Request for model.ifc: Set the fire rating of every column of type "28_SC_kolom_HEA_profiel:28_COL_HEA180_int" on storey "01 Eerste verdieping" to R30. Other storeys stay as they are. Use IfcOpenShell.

First a look at what the model holds.

```python
import ifcopenshell
import ifcopenshell.util.element

model = ifcopenshell.open("model.ifc")
print(model.schema)
storey = next(s for s in model.by_type("IfcBuildingStorey") if s.Name == "01 Eerste verdieping")
columns = [e for e in ifcopenshell.util.element.get_decomposition(storey) if e.is_a("IfcColumn")]
seen = {}
for e in columns:
    element_type = ifcopenshell.util.element.get_type(e)
    key = (element_type.Name if element_type != e and element_type else None, ifcopenshell.util.element.get_pset(e, "Pset_ColumnCommon", "FireRating"))
    seen[key] = seen.get(key, 0) + 1
for (name, value), count in sorted(seen.items(), key=str):
    print(count, "x", name, "|", value)
```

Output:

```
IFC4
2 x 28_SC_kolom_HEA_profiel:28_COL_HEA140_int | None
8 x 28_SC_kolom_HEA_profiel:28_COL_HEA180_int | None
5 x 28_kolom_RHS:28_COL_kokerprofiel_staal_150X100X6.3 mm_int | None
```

```python
import ifcopenshell
import ifcopenshell.api.pset
import ifcopenshell.util.element

model = ifcopenshell.open("model.ifc")

storey = next(s for s in model.by_type("IfcBuildingStorey") if s.Name == "01 Eerste verdieping")
columns = [e for e in ifcopenshell.util.element.get_decomposition(storey) if e.is_a("IfcColumn")]

count = 0
for e in columns:
    element_type = ifcopenshell.util.element.get_type(e)
    if element_type in (None, e) or element_type.Name != "28_SC_kolom_HEA_profiel:28_COL_HEA180_int":
        continue
    # add_pset returns the element's existing set when there is one.
    pset = ifcopenshell.api.pset.add_pset(model, product=e, name="Pset_ColumnCommon")
    ifcopenshell.api.pset.edit_pset(model, pset=pset, properties={"FireRating": "R30"})
    count += 1

print(count, "columns updated")

model.write("model_rev.ifc")
```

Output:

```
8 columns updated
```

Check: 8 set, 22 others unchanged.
